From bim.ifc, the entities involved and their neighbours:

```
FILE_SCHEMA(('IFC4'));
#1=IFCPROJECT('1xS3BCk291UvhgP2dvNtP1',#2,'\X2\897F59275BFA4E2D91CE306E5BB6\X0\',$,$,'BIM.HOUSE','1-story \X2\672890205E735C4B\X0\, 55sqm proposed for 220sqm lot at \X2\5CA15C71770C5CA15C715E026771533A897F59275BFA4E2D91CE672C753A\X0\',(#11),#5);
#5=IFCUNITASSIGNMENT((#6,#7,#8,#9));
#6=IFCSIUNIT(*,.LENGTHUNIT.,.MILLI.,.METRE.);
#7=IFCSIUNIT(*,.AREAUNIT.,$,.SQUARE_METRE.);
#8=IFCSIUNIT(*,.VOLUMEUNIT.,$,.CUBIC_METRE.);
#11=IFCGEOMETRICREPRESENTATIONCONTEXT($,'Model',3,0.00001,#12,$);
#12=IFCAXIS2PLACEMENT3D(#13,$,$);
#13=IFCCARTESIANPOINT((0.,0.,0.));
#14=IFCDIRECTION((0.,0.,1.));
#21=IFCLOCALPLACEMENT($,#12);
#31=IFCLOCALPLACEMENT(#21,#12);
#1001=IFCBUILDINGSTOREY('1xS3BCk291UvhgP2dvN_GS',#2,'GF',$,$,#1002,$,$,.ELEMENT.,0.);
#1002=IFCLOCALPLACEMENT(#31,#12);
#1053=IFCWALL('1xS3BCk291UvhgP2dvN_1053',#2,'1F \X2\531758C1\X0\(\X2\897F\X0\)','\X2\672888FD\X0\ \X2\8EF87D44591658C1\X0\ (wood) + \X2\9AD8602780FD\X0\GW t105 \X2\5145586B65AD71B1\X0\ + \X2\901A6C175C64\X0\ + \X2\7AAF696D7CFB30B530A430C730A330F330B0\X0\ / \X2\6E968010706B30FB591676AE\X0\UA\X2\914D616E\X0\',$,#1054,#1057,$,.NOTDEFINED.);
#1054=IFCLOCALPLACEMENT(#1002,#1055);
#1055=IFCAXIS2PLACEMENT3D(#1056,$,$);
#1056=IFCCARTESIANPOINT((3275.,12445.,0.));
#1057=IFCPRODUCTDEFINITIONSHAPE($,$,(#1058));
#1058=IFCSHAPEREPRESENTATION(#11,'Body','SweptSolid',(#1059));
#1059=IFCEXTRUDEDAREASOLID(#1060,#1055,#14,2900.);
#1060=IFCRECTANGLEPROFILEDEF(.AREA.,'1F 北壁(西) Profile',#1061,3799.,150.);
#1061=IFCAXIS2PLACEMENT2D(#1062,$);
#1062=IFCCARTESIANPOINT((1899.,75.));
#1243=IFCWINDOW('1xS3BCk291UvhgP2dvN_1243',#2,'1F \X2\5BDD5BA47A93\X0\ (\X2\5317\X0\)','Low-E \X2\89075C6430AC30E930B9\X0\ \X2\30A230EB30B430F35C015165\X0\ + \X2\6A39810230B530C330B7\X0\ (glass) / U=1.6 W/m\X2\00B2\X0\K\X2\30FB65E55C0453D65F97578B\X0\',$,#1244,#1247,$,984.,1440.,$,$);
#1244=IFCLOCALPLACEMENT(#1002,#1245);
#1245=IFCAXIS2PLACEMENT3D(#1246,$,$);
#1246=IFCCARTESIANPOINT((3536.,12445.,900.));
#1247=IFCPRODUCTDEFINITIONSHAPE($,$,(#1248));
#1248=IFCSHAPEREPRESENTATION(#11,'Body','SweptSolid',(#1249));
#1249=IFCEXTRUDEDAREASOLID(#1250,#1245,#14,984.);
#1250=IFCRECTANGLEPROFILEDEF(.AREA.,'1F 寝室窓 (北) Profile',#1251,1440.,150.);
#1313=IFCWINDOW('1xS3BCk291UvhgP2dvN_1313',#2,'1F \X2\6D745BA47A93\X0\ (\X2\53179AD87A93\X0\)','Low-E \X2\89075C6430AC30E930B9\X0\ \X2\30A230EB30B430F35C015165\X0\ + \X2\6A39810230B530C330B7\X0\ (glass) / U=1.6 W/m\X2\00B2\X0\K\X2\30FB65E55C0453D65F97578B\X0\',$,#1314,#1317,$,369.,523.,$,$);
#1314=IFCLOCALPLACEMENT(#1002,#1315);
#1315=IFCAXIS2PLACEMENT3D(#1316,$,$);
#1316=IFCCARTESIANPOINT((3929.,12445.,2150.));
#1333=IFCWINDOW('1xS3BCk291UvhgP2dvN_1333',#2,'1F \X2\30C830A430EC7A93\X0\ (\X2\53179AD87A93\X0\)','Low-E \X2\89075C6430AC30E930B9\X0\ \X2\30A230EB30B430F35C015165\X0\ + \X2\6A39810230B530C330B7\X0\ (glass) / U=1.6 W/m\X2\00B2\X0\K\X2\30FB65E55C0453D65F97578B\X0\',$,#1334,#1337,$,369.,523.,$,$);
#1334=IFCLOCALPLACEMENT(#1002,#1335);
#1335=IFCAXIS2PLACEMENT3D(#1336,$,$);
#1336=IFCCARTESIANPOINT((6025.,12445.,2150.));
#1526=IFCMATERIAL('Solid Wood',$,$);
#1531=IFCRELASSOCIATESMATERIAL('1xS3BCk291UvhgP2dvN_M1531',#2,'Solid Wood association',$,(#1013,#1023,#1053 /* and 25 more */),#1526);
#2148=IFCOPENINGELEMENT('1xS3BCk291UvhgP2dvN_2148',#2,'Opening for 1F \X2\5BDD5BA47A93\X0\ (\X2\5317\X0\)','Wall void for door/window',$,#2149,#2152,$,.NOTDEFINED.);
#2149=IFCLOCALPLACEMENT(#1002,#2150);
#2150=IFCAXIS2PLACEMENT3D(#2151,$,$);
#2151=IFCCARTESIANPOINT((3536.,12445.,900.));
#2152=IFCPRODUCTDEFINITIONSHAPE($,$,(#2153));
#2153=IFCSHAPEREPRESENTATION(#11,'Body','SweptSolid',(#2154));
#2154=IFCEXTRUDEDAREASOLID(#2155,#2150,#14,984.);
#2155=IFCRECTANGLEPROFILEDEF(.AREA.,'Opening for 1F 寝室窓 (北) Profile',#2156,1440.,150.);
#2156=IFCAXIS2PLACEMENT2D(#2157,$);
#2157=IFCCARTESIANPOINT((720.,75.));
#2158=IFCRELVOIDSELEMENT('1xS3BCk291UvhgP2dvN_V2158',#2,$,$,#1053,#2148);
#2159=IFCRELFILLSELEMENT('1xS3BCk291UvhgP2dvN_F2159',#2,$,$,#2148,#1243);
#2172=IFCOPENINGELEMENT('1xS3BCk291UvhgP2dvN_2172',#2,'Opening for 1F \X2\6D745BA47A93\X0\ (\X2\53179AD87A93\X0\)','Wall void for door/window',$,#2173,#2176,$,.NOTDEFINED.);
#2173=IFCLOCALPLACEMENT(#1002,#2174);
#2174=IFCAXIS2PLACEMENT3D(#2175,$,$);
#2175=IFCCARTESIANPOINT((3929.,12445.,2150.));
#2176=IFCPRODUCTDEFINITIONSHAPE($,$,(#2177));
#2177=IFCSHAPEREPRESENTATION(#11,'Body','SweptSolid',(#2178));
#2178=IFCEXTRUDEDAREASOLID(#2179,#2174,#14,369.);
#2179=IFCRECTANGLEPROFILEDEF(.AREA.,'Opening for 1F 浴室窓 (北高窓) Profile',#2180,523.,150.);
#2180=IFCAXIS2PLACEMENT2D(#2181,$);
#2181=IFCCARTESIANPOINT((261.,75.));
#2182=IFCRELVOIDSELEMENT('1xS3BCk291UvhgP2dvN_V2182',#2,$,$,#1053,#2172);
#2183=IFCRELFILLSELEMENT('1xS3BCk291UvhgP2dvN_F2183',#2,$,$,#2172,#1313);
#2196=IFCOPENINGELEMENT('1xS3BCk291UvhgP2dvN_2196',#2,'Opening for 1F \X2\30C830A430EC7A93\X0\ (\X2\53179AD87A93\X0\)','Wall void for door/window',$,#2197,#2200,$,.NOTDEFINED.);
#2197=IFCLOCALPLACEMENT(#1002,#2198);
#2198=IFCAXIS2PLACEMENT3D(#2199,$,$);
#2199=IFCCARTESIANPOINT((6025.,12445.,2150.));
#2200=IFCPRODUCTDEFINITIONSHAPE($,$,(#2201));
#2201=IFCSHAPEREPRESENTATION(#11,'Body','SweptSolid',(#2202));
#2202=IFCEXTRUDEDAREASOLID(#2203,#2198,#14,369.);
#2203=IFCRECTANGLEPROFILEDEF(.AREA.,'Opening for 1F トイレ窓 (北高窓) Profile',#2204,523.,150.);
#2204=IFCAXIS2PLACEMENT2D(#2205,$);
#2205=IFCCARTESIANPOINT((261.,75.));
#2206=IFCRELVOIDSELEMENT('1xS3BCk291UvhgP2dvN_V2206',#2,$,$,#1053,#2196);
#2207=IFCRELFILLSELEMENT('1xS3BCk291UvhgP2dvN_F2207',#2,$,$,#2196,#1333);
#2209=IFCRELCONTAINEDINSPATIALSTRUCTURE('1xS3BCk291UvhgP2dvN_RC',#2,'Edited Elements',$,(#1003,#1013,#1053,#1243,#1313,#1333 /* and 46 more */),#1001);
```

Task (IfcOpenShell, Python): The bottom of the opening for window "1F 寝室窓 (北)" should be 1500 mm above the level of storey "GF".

```python
import numpy as np
import ifcopenshell
import ifcopenshell.api.geometry
import ifcopenshell.geom
import ifcopenshell.util.element
import ifcopenshell.util.placement
import ifcopenshell.util.shape
import ifcopenshell.util.unit

model = ifcopenshell.open("bim.ifc")
unit_scale = ifcopenshell.util.unit.calculate_unit_scale(model)

window = model.by_id(1243)
opening = window.FillsVoids[0].RelatingOpeningElement
storey = ifcopenshell.util.element.get_container(window, ifc_class="IfcBuildingStorey")
level = ifcopenshell.util.placement.get_local_placement(storey.ObjectPlacement)[2, 3]

# The opening's origin need not be at the sill, so measure its lowest point.
shape = ifcopenshell.geom.create_shape(ifcopenshell.geom.settings(), opening)
bottom = ifcopenshell.util.shape.get_shape_bottom_elevation(shape, shape.geometry) / unit_scale
dz = level + 1.5 / unit_scale - bottom

shift = np.array([0.0, 0.0, dz])
# The window is not placed relative to its opening, so move both.
for product in (opening, window):
    matrix = ifcopenshell.util.placement.get_local_placement(product.ObjectPlacement)
    matrix[:3, 3] += shift
    ifcopenshell.api.geometry.edit_object_placement(model, product=product, matrix=matrix, is_si=False)

print(f"moved by {dz * unit_scale:+.3f} m")

model.write("bim_edited.ifc")
```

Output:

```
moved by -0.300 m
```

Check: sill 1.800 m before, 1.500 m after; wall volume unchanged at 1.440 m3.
